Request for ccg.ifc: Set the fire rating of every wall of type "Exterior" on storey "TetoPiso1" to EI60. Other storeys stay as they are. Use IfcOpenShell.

First a look at what the model holds.

```python
import ifcopenshell
import ifcopenshell.util.element

model = ifcopenshell.open("ccg.ifc")
print(model.schema)
storey = next(s for s in model.by_type("IfcBuildingStorey") if s.Name == "TetoPiso1")
walls = [e for e in ifcopenshell.util.element.get_decomposition(storey) if e.is_a("IfcWall")]
seen = {}
for e in walls:
    element_type = ifcopenshell.util.element.get_type(e)
    key = (element_type.Name if element_type != e and element_type else None, ifcopenshell.util.element.get_pset(e, "Pset_WallCommon", "FireRating"))
    seen[key] = seen.get(key, 0) + 1
for (name, value), count in sorted(seen.items(), key=str):
    print(count, "x", name, "|", value)
```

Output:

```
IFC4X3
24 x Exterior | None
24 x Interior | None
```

```python
import ifcopenshell
import ifcopenshell.api.pset
import ifcopenshell.util.element

model = ifcopenshell.open("ccg.ifc")

storey = next(s for s in model.by_type("IfcBuildingStorey") if s.Name == "TetoPiso1")
walls = [e for e in ifcopenshell.util.element.get_decomposition(storey) if e.is_a("IfcWall")]

count = 0
for e in walls:
    element_type = ifcopenshell.util.element.get_type(e)
    if element_type in (None, e) or element_type.Name != "Exterior":
        continue
    # add_pset returns the element's existing set when there is one.
    pset = ifcopenshell.api.pset.add_pset(model, product=e, name="Pset_WallCommon")
    ifcopenshell.api.pset.edit_pset(model, pset=pset, properties={"FireRating": "EI60"})
    count += 1

print(count, "walls updated")

model.write("ccg_edited.ifc")
```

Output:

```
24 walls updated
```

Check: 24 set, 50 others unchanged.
